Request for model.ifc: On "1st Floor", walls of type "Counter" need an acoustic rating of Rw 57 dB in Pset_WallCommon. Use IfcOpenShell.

First a look at what the model holds.

```python
import ifcopenshell
import ifcopenshell.util.element

model = ifcopenshell.open("model.ifc")
print(model.schema)
storey = next(s for s in model.by_type("IfcBuildingStorey") if s.Name == "1st Floor")
walls = [e for e in ifcopenshell.util.element.get_decomposition(storey) if e.is_a("IfcWall")]
seen = {}
for e in walls:
    element_type = ifcopenshell.util.element.get_type(e)
    key = (element_type.Name if element_type != e and element_type else None, ifcopenshell.util.element.get_pset(e, "Pset_WallCommon", "AcousticRating"))
    seen[key] = seen.get(key, 0) + 1
for (name, value), count in sorted(seen.items(), key=str):
    print(count, "x", name, "|", value)
```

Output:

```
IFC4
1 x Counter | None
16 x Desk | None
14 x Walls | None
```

```python
import ifcopenshell
import ifcopenshell.api.pset
import ifcopenshell.util.element

model = ifcopenshell.open("model.ifc")

storey = next(s for s in model.by_type("IfcBuildingStorey") if s.Name == "1st Floor")
walls = [e for e in ifcopenshell.util.element.get_decomposition(storey) if e.is_a("IfcWall")]

count = 0
for e in walls:
    element_type = ifcopenshell.util.element.get_type(e)
    if element_type in (None, e) or element_type.Name != "Counter":
        continue
    # add_pset returns the element's existing set when there is one.
    pset = ifcopenshell.api.pset.add_pset(model, product=e, name="Pset_WallCommon")
    ifcopenshell.api.pset.edit_pset(model, pset=pset, properties={"AcousticRating": "Rw 57 dB"})
    count += 1

print(count, "walls updated")

model.write("model-out.ifc")
```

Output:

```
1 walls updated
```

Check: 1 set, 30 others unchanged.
